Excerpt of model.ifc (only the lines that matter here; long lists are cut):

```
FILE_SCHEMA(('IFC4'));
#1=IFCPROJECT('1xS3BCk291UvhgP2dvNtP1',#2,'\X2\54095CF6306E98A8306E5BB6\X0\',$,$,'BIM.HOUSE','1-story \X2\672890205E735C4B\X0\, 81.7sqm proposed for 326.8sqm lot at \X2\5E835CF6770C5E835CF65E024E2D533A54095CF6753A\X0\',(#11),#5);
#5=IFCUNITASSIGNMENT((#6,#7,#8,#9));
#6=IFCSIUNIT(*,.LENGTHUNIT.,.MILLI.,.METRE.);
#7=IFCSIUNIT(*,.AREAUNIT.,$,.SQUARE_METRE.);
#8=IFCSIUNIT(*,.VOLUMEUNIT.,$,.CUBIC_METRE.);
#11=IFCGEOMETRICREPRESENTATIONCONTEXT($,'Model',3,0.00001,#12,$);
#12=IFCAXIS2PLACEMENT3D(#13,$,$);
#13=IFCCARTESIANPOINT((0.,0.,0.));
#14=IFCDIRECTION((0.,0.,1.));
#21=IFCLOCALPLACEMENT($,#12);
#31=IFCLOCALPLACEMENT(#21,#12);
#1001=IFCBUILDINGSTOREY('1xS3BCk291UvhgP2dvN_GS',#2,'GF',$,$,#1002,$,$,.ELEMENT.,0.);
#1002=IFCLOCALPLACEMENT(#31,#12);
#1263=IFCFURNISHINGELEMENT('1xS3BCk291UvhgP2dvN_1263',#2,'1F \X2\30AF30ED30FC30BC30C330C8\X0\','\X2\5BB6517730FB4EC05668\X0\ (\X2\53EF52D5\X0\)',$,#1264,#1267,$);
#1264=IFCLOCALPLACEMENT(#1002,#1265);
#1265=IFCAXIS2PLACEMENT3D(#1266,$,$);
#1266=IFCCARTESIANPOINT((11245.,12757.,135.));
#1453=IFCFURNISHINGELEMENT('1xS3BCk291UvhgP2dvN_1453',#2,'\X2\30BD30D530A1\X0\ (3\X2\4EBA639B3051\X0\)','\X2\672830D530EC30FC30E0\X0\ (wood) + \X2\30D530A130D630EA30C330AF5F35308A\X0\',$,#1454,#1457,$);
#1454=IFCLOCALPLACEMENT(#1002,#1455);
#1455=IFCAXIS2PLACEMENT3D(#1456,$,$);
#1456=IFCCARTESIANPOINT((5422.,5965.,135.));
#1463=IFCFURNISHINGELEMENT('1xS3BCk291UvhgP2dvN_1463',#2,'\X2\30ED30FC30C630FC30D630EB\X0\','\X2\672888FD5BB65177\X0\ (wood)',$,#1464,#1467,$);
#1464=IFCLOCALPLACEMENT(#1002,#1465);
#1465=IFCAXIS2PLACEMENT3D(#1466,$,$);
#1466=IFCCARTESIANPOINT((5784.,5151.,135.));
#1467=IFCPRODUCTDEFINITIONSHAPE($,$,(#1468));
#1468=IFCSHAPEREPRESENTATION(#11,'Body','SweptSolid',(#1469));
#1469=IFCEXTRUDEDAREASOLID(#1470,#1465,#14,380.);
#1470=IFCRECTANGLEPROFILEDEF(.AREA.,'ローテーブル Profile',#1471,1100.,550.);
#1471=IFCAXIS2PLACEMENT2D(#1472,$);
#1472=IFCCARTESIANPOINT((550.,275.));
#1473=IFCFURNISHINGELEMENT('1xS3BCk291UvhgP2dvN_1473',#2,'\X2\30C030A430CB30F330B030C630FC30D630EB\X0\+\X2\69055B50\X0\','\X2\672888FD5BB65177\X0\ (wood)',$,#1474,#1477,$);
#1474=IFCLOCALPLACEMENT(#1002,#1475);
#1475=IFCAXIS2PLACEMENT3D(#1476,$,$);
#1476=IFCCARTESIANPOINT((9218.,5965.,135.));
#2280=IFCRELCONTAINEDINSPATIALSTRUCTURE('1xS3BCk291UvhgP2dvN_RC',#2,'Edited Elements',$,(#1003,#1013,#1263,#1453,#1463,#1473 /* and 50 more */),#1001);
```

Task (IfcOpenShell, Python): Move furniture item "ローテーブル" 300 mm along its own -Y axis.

```python
import ifcopenshell
import ifcopenshell.api.geometry
import ifcopenshell.util.placement
import ifcopenshell.util.unit

model = ifcopenshell.open("model.ifc")
unit_scale = ifcopenshell.util.unit.calculate_unit_scale(model)

item = model.by_id(1463)
matrix = ifcopenshell.util.placement.get_local_placement(item.ObjectPlacement)
matrix[:3, 3] -= matrix[:3, 1] * 0.3 / unit_scale
ifcopenshell.api.geometry.edit_object_placement(model, product=item, matrix=matrix, is_si=False)

print(ifcopenshell.util.placement.get_local_placement(item.ObjectPlacement).round(3) + 0.0)

model.write("model-out.ifc")
```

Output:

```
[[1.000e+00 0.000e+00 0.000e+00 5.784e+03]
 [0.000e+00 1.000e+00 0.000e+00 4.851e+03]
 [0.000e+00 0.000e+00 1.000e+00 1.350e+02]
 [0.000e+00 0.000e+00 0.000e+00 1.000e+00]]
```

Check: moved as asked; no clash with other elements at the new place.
